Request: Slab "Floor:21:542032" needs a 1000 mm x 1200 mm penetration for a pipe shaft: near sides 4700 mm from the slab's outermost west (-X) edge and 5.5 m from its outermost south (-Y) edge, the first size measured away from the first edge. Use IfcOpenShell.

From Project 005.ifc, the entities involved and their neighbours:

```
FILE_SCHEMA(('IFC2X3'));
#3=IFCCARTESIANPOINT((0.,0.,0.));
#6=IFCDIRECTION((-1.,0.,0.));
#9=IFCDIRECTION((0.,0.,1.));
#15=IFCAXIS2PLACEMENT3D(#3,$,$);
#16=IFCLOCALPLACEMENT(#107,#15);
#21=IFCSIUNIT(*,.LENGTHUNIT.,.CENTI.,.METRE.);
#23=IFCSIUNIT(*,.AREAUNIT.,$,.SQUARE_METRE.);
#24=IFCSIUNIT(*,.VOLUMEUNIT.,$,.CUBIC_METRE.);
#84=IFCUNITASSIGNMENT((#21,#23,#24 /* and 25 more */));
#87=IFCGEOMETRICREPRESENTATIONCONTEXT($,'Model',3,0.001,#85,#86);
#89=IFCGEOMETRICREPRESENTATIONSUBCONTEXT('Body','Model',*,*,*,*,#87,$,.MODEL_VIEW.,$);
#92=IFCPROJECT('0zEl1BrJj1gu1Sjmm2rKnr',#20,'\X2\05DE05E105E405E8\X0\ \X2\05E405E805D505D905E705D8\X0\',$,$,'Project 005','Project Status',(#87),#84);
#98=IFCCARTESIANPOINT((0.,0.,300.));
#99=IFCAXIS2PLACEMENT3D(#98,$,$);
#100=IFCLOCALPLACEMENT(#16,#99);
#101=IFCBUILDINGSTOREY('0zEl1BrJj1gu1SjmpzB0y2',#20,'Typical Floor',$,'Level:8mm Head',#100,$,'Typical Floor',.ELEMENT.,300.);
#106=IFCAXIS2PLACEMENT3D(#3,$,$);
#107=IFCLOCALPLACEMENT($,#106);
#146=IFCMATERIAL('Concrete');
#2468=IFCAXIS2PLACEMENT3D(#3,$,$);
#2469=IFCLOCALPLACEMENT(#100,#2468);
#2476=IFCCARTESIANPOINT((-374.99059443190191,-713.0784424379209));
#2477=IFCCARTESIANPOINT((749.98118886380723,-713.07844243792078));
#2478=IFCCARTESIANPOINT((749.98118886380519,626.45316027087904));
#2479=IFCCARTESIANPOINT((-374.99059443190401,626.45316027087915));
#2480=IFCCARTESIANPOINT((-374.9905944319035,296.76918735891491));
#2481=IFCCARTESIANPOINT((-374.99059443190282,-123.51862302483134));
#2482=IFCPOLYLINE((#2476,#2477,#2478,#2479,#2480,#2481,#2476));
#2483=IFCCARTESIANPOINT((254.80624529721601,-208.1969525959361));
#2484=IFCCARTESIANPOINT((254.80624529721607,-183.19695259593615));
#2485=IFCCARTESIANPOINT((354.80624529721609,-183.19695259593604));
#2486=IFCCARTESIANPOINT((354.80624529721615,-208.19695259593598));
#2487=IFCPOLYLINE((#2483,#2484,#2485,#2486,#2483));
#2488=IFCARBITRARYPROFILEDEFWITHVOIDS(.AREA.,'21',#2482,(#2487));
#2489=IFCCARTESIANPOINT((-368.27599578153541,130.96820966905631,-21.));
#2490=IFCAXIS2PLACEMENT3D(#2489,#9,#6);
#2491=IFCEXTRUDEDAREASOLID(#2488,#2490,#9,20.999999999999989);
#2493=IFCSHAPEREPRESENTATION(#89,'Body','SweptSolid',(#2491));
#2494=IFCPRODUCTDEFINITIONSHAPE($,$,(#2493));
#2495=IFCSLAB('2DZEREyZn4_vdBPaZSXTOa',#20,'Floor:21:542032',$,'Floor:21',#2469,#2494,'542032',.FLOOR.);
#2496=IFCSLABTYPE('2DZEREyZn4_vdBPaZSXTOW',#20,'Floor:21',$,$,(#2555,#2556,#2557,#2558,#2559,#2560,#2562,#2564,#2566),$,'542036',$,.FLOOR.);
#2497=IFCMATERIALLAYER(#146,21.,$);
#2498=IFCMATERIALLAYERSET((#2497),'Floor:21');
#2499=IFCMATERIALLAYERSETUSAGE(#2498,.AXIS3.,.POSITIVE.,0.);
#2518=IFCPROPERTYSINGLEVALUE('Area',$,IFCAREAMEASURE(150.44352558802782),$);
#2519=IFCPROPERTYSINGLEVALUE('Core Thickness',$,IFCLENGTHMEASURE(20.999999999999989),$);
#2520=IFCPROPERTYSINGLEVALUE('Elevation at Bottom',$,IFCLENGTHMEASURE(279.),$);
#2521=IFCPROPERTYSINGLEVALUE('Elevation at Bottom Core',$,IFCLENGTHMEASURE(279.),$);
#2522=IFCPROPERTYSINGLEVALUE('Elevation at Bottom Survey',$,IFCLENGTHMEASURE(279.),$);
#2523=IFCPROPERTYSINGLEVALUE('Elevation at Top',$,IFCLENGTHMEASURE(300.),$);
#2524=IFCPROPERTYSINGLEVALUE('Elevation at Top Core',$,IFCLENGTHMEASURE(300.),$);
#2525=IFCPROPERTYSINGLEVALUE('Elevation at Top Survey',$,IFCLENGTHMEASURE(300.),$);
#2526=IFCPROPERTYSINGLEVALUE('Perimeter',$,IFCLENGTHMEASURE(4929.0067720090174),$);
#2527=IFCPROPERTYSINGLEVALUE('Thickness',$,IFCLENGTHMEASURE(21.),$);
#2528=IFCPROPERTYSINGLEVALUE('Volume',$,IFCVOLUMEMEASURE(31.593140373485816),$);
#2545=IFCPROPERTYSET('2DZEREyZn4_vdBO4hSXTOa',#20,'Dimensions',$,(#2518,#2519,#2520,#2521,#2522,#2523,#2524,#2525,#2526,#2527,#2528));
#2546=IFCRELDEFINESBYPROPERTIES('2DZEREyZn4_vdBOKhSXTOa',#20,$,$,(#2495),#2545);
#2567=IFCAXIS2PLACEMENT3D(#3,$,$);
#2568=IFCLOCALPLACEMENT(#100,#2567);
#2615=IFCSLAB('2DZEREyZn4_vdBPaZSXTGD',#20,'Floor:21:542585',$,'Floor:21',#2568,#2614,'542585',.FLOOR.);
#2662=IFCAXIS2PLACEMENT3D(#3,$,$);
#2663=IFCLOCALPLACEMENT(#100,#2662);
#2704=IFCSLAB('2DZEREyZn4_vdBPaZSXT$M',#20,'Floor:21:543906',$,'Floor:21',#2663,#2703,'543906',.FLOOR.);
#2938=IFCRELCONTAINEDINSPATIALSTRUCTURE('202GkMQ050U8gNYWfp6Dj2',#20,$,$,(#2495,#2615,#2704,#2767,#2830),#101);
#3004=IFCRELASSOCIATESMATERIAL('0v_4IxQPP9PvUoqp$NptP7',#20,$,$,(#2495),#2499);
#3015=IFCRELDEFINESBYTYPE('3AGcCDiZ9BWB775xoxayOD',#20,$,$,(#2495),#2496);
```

```python
import numpy as np
import ifcopenshell
import ifcopenshell.api.feature
import ifcopenshell.api.geometry
import ifcopenshell.api.pset
import ifcopenshell.api.root
import ifcopenshell.geom
import ifcopenshell.util.element
import ifcopenshell.util.placement
import ifcopenshell.util.representation
import ifcopenshell.util.shape
import ifcopenshell.util.unit

model = ifcopenshell.open("Project 005.ifc")
unit_scale = ifcopenshell.util.unit.calculate_unit_scale(model)
area_scale = ifcopenshell.util.unit.calculate_unit_scale(model, "AREAUNIT")
volume_scale = ifcopenshell.util.unit.calculate_unit_scale(model, "VOLUMEUNIT")
settings = ifcopenshell.geom.settings()


def volume(element):
    """Net volume in cubic metres, openings subtracted."""
    shape = ifcopenshell.geom.create_shape(settings, element)
    return ifcopenshell.util.shape.get_volume(shape.geometry)


slab = model.by_guid("2DZEREyZn4_vdBPaZSXTOa")
before = volume(slab)

# Extent in the slab's own axes, in metres. The edges named are its -X and -Y sides.
slab_shape = ifcopenshell.geom.create_shape(settings, slab)
vertices = ifcopenshell.util.shape.get_vertices(slab_shape.geometry)
x_min, y_min, bottom = vertices.min(axis=0)
top = vertices[:, 2].max()

opening = ifcopenshell.api.root.create_entity(model, ifc_class="IfcOpeningElement", name="Pipe shaft opening")
context = ifcopenshell.util.representation.get_context(model, "Model", "Body", "MODEL_VIEW")
width, depth = 1, 1.2
outline = [(0.0, 0.0), (width, 0.0), (width, depth), (0.0, depth), (0.0, 0.0)]
# Overshoot both faces by 50 mm so the cut is clean.
shape = ifcopenshell.api.geometry.add_slab_representation(
    model, context=context, depth=top - bottom + 0.1, polyline=outline
)
ifcopenshell.api.geometry.assign_representation(model, product=opening, representation=shape)

matrix = ifcopenshell.util.placement.get_local_placement(slab.ObjectPlacement)
matrix[:, 3] = matrix @ np.append(np.array([x_min + 4.7, y_min + 5.5, bottom - 0.05]) / unit_scale, 1.0)
ifcopenshell.api.geometry.edit_object_placement(model, product=opening, matrix=matrix, is_si=False)
ifcopenshell.api.feature.add_feature(model, feature=opening, element=slab)

after = volume(slab)

# Update the slab's stored quantities.
pset = model.by_id(ifcopenshell.util.element.get_pset(slab, "Dimensions", should_inherit=False)["id"])
ifcopenshell.api.pset.edit_pset(model, pset=pset, properties={
    "Area": model.create_entity("IfcAreaMeasure", after / (top - bottom) / area_scale),
    "Volume": model.create_entity("IfcVolumeMeasure", after / volume_scale),
})

print(f"slab volume {before:.3f} -> {after:.3f} m3")

model.write("Project 005-out.ifc")
```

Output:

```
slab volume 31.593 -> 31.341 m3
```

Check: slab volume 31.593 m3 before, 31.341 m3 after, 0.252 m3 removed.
